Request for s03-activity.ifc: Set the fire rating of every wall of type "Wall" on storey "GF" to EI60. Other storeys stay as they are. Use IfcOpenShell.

First a look at what the model holds.

```python
import ifcopenshell
import ifcopenshell.util.element

model = ifcopenshell.open("s03-activity.ifc")
print(model.schema)
storey = next(s for s in model.by_type("IfcBuildingStorey") if s.Name == "GF")
walls = [e for e in ifcopenshell.util.element.get_decomposition(storey) if e.is_a("IfcWall")]
seen = {}
for e in walls:
    element_type = ifcopenshell.util.element.get_type(e)
    key = (element_type.Name if element_type != e and element_type else None, ifcopenshell.util.element.get_pset(e, "Pset_WallCommon", "FireRating"))
    seen[key] = seen.get(key, 0) + 1
for (name, value), count in sorted(seen.items(), key=str):
    print(count, "x", name, "|", value)
```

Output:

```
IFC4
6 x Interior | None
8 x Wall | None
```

```python
import ifcopenshell
import ifcopenshell.api.pset
import ifcopenshell.util.element

model = ifcopenshell.open("s03-activity.ifc")

storey = next(s for s in model.by_type("IfcBuildingStorey") if s.Name == "GF")
walls = [e for e in ifcopenshell.util.element.get_decomposition(storey) if e.is_a("IfcWall")]

count = 0
for e in walls:
    element_type = ifcopenshell.util.element.get_type(e)
    if element_type in (None, e) or element_type.Name != "Wall":
        continue
    # add_pset returns the element's existing set when there is one.
    pset = ifcopenshell.api.pset.add_pset(model, product=e, name="Pset_WallCommon")
    ifcopenshell.api.pset.edit_pset(model, pset=pset, properties={"FireRating": "EI60"})
    count += 1

print(count, "walls updated")

model.write("s03-activity_rev.ifc")
```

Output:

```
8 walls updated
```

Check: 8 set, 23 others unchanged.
